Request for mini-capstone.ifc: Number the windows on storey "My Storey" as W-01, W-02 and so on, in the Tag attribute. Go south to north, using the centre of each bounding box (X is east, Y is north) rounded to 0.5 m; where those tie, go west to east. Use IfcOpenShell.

First a look at what the model holds.

```python
import ifcopenshell
import ifcopenshell.util.element
import ifcopenshell.util.placement

model = ifcopenshell.open("mini-capstone.ifc")
print(model.schema)
storey = next(s for s in model.by_type("IfcBuildingStorey") if s.Name == "My Storey")
windows = [e for e in ifcopenshell.util.element.get_decomposition(storey) if e.is_a("IfcWindow")]
for e in sorted(windows, key=lambda e: e.id()):
    origin = ifcopenshell.util.placement.get_local_placement(e.ObjectPlacement)[:3, 3]
    print(e.id(), e.Tag, e.Name, origin.round(2) + 0.0, sep=" | ")
```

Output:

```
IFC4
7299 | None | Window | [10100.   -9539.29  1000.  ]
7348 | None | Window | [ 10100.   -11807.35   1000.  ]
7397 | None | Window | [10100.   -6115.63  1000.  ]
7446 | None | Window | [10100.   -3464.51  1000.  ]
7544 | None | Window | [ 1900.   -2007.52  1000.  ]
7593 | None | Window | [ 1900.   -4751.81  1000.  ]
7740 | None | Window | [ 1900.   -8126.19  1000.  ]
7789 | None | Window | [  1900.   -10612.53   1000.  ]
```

```python
import ifcopenshell
import ifcopenshell.geom
import ifcopenshell.util.element
import ifcopenshell.util.shape

model = ifcopenshell.open("mini-capstone.ifc")
settings = ifcopenshell.geom.settings()
settings.set("use-world-coords", True)


def centre(element):
    shape = ifcopenshell.geom.create_shape(settings, element)
    return ifcopenshell.util.shape.get_bbox_centroid(shape.geometry)


storey = next(s for s in model.by_type("IfcBuildingStorey") if s.Name == "My Storey")
windows = [e for e in ifcopenshell.util.element.get_decomposition(storey) if e.is_a("IfcWindow")]

# Insertion points can sit at a corner or the storey origin, so sort by the geometry (in metres).
centres = {e: centre(e) for e in windows}
windows.sort(key=lambda e: (round(centres[e][1] / 0.5), centres[e][0]))

for i, e in enumerate(windows, start=1):
    number = f"W-{i:02d}"
    e.Tag = number
    print(e.id(), number)

model.write("mini-capstone-out.ifc")
```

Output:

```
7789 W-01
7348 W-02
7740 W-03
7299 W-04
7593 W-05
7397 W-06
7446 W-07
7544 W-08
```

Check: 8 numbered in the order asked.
